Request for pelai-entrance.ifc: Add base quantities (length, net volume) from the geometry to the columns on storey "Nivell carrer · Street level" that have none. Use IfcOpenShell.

First a look at what the model holds.

```python
import ifcopenshell
import ifcopenshell.util.element
import ifcopenshell.util.unit

model = ifcopenshell.open("pelai-entrance.ifc")
print(model.schema)
for unit_type in ("LENGTHUNIT", "AREAUNIT", "VOLUMEUNIT"):
    print(unit_type, ifcopenshell.util.unit.calculate_unit_scale(model, unit_type))
storey = next(s for s in model.by_type("IfcBuildingStorey") if s.Name == "Nivell carrer · Street level")
columns = [e for e in ifcopenshell.util.element.get_decomposition(storey) if e.is_a("IfcColumn")]
for e in sorted(columns, key=lambda e: e.id()):
    print(e.id(), e.is_a(), e.Name, list(ifcopenshell.util.element.get_psets(e, qtos_only=True)), sep=" | ")
```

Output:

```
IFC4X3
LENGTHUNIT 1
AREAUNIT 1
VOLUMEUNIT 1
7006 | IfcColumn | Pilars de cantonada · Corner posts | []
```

```python
import ifcopenshell
import ifcopenshell.api.pset
import ifcopenshell.geom
import ifcopenshell.util.element
import ifcopenshell.util.shape
import ifcopenshell.util.unit

model = ifcopenshell.open("pelai-entrance.ifc")
unit_scale = ifcopenshell.util.unit.calculate_unit_scale(model)
volume_scale = ifcopenshell.util.unit.calculate_unit_scale(model, "VOLUMEUNIT")
settings = ifcopenshell.geom.settings()

storey = next(s for s in model.by_type("IfcBuildingStorey") if s.Name == "Nivell carrer · Street level")
columns = [e for e in ifcopenshell.util.element.get_decomposition(storey) if e.is_a("IfcColumn")]

for e in sorted(columns, key=lambda e: e.id()):
    if ifcopenshell.util.element.get_psets(e, qtos_only=True, should_inherit=False):
        continue
    # Geometry comes back in metres, in the element's own axes.
    shape = ifcopenshell.geom.create_shape(settings, e)
    values = {
        "Length": ifcopenshell.util.shape.get_z(shape.geometry) / unit_scale,
        "NetVolume": ifcopenshell.util.shape.get_volume(shape.geometry) / volume_scale,
    }
    qto = ifcopenshell.api.pset.add_qto(model, product=e, name="Qto_ColumnBaseQuantities")
    ifcopenshell.api.pset.edit_qto(model, qto=qto, properties=values)
    print(e.id(), {k: round(v, 3) for k, v in values.items()})

model.write("pelai-entrance-out.ifc")
```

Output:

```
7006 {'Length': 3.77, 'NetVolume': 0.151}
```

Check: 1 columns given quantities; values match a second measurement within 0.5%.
